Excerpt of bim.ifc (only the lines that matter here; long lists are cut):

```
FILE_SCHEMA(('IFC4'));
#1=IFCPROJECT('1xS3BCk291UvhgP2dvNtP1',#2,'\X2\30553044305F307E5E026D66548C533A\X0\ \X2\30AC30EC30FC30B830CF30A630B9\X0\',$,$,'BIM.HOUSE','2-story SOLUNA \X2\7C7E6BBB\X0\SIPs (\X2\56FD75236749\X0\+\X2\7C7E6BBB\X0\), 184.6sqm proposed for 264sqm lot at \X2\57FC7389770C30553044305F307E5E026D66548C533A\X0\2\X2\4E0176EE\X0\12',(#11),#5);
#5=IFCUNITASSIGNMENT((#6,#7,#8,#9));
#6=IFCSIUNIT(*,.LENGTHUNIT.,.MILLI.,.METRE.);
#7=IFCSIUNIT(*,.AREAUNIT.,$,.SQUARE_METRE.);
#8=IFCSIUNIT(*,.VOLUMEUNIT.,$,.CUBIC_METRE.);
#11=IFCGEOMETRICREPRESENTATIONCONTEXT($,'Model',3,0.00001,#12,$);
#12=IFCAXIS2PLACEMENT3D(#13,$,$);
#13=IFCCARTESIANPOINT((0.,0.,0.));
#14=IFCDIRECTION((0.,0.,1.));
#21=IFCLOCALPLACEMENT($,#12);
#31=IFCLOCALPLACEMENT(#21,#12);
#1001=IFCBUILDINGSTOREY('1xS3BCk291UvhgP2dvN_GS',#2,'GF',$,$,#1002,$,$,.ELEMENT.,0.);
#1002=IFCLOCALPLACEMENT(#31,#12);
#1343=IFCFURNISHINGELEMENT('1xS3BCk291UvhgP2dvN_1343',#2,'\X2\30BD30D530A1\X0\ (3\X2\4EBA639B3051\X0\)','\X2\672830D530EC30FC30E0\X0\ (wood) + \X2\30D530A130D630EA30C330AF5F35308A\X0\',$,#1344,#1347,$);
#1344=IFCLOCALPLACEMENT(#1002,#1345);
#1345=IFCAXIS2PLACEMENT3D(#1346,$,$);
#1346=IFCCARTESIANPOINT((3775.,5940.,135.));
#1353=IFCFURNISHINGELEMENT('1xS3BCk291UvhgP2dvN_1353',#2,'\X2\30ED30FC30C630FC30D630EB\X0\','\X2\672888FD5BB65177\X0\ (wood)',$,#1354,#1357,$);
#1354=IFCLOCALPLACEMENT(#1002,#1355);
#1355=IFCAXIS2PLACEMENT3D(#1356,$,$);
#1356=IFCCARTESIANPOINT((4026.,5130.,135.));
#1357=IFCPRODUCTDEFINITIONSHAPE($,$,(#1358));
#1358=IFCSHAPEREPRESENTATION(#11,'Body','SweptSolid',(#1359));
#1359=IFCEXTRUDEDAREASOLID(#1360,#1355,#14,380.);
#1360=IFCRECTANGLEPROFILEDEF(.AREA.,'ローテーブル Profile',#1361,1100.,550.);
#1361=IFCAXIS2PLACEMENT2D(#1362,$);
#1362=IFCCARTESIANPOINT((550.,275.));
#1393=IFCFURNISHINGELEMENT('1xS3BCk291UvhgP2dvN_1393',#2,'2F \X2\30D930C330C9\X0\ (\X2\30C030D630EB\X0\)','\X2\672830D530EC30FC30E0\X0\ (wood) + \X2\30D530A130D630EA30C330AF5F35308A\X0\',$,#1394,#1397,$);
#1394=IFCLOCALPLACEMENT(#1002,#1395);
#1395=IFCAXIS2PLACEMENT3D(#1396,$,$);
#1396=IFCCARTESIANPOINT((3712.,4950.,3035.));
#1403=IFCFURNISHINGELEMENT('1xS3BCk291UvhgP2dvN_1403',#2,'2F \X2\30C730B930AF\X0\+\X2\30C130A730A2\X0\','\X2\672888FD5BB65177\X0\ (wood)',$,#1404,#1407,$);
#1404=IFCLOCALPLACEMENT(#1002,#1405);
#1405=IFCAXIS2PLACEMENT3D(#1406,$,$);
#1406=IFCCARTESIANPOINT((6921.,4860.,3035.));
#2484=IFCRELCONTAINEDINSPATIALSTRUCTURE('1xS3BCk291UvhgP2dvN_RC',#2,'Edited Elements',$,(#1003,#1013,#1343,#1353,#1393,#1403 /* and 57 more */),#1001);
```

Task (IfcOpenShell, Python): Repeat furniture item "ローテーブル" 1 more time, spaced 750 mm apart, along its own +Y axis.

```python
import ifcopenshell
import ifcopenshell.api.geometry
import ifcopenshell.api.root
import ifcopenshell.util.element
import ifcopenshell.util.placement

model = ifcopenshell.open("bim.ifc")


def reuse_history(source, copy):
    """copy_class also copies each property set's owner history, people and application; keep the originals."""
    for rel in copy.IsDefinedBy:
        if rel.is_a("IfcRelDefinesByProperties") and (history := rel.RelatingPropertyDefinition.OwnerHistory):
            rel.RelatingPropertyDefinition.OwnerHistory = source.OwnerHistory
            ifcopenshell.util.element.remove_deep2(model, history)


source = model.by_guid("1xS3BCk291UvhgP2dvN_1353")
base = ifcopenshell.util.placement.get_local_placement(source.ObjectPlacement)
step = base[:3, 1] * 750.0

for i in range(1, 2):
    copy = ifcopenshell.api.root.copy_class(model, product=source)
    copy.Representation = ifcopenshell.util.element.copy_deep(
        model, source.Representation, exclude=["IfcGeometricRepresentationContext", "IfcRepresentationMap"]
    )
    reuse_history(source, copy)
    matrix = base.copy()
    matrix[:3, 3] += i * step
    print("added at", matrix[:3, 3].round(3) + 0.0)
    ifcopenshell.api.geometry.edit_object_placement(model, product=copy, matrix=matrix, is_si=False)

model.write("bim_rev.ifc")
```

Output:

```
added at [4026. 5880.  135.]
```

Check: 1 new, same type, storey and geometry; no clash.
